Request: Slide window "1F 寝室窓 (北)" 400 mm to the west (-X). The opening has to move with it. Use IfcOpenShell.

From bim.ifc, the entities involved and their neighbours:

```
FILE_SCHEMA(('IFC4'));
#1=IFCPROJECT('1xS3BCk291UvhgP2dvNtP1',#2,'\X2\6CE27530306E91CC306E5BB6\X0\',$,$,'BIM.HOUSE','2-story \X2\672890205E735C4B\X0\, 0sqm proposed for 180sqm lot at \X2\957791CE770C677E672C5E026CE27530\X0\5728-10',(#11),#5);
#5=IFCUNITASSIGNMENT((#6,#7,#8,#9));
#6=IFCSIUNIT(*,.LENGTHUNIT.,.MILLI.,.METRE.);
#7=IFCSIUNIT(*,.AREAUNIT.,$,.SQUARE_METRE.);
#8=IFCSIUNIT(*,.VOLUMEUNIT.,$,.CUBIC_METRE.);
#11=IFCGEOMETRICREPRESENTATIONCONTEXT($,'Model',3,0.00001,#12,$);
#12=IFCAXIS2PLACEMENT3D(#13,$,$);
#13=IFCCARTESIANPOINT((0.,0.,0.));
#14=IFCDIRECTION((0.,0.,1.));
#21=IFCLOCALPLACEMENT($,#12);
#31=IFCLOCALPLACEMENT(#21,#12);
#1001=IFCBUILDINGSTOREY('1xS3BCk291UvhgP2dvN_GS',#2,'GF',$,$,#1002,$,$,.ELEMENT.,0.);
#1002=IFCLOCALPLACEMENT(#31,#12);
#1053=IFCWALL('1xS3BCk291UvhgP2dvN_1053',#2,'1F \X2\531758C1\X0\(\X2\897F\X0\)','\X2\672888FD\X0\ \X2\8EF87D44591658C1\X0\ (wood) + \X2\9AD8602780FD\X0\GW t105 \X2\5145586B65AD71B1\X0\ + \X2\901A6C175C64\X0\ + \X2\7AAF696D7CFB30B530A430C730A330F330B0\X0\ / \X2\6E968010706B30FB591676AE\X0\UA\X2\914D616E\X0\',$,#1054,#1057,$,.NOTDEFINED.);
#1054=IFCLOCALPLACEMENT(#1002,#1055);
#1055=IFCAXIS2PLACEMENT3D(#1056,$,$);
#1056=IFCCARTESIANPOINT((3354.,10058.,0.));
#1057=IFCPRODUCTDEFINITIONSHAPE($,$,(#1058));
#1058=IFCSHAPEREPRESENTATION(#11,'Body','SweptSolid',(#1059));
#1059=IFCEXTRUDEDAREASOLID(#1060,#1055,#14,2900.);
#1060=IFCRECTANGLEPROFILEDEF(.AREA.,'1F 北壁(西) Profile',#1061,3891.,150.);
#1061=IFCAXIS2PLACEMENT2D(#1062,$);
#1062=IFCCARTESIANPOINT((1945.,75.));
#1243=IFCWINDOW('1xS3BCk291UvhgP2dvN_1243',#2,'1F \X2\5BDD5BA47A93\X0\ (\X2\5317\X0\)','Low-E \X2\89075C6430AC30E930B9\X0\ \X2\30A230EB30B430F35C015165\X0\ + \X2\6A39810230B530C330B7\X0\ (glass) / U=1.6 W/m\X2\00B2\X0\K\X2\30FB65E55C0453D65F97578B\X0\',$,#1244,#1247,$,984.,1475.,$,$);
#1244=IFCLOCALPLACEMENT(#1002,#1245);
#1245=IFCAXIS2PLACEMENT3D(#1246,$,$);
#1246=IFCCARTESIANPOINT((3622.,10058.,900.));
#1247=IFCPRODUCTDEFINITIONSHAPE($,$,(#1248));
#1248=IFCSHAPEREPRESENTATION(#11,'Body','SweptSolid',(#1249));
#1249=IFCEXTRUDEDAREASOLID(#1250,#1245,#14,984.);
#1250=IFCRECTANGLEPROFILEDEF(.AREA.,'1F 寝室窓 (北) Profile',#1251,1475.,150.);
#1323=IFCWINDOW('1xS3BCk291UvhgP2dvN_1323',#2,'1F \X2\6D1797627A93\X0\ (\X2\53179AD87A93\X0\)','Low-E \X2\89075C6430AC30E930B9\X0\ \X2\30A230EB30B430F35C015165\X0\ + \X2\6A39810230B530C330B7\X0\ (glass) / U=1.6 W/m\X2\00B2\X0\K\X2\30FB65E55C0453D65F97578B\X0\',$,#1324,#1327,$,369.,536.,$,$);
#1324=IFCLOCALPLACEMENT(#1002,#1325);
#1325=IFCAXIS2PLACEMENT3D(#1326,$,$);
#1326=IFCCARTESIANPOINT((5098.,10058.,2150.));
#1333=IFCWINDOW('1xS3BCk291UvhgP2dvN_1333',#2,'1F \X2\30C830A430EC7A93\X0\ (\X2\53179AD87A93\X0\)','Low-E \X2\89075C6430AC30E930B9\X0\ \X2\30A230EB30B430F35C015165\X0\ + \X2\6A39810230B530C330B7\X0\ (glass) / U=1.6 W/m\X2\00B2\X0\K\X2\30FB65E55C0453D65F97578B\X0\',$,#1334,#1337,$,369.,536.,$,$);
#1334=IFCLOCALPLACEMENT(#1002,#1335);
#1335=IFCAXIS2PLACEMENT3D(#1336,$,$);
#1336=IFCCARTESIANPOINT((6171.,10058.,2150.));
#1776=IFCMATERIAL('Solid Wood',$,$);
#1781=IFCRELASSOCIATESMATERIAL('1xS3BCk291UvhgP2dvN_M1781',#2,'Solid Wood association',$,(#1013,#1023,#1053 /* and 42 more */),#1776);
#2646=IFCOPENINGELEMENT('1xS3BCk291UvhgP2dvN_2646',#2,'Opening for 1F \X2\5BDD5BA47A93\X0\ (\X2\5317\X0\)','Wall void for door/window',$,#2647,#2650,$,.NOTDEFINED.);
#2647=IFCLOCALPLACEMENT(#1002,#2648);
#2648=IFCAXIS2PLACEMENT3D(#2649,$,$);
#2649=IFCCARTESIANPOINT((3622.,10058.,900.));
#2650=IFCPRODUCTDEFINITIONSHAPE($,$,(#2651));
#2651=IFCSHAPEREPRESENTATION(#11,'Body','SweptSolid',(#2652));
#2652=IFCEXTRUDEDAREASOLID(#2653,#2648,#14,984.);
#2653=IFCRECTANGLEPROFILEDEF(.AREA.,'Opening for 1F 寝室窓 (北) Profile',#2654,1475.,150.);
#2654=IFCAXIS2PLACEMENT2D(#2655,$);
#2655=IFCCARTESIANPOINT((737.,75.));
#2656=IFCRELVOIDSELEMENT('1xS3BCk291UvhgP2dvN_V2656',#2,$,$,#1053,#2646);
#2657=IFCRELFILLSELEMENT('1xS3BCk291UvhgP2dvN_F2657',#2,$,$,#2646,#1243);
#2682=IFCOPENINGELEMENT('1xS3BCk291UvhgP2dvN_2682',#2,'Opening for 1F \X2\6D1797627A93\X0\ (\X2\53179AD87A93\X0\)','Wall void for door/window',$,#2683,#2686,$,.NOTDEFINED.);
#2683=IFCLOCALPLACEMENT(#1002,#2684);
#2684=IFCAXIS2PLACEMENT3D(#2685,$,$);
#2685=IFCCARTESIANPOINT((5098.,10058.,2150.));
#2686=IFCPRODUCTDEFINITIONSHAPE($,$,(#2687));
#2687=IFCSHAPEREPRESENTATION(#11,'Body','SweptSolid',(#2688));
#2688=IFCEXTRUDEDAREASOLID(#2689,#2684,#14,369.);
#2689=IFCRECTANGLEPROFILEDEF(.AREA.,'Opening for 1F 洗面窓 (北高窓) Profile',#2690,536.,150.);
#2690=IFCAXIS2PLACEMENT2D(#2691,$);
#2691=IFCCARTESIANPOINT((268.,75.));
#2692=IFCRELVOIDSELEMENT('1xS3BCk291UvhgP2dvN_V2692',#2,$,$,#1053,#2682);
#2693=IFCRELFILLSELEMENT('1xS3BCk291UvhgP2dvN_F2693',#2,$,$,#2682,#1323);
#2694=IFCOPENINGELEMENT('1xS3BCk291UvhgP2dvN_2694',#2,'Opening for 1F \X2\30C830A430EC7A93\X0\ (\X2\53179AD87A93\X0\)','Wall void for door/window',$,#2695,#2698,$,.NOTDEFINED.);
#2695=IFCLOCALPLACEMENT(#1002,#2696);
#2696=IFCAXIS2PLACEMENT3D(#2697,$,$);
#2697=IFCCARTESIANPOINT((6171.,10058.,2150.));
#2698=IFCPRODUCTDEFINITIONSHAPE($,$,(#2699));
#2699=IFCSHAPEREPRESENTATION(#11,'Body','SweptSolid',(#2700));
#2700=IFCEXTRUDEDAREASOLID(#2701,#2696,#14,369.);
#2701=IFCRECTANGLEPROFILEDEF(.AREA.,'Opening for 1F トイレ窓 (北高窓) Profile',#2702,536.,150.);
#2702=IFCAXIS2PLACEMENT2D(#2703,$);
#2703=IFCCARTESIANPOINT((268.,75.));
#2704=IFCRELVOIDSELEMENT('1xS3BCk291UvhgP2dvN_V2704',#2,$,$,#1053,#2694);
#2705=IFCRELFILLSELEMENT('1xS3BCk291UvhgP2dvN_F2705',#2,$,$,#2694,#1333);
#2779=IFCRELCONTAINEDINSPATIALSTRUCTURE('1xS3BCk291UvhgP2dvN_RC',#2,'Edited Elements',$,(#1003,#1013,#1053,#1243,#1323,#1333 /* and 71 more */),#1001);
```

```python
import ifcopenshell
import ifcopenshell.api.geometry
import ifcopenshell.util.placement
import ifcopenshell.util.unit

model = ifcopenshell.open("bim.ifc")
unit_scale = ifcopenshell.util.unit.calculate_unit_scale(model)

window = model.by_id(1243)
opening = window.FillsVoids[0].RelatingOpeningElement
wall = opening.VoidsElements[0].RelatingBuildingElement

wall_matrix = ifcopenshell.util.placement.get_local_placement(wall.ObjectPlacement)
shift = wall_matrix[:3, 0] * -0.4 / unit_scale
before = ifcopenshell.util.placement.get_local_placement(window.ObjectPlacement)[:3, 3].copy()

# The window is not placed relative to its opening, so move both.
for product in (opening, window):
    matrix = ifcopenshell.util.placement.get_local_placement(product.ObjectPlacement)
    matrix[:3, 3] += shift
    ifcopenshell.api.geometry.edit_object_placement(model, product=product, matrix=matrix, is_si=False)

after = ifcopenshell.util.placement.get_local_placement(window.ObjectPlacement)[:3, 3]
print("window moved by", (after - before).round(3) + 0.0)

model.write("bim-out.ifc")
```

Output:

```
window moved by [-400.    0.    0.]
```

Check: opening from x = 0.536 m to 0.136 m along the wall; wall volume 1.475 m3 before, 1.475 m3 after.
